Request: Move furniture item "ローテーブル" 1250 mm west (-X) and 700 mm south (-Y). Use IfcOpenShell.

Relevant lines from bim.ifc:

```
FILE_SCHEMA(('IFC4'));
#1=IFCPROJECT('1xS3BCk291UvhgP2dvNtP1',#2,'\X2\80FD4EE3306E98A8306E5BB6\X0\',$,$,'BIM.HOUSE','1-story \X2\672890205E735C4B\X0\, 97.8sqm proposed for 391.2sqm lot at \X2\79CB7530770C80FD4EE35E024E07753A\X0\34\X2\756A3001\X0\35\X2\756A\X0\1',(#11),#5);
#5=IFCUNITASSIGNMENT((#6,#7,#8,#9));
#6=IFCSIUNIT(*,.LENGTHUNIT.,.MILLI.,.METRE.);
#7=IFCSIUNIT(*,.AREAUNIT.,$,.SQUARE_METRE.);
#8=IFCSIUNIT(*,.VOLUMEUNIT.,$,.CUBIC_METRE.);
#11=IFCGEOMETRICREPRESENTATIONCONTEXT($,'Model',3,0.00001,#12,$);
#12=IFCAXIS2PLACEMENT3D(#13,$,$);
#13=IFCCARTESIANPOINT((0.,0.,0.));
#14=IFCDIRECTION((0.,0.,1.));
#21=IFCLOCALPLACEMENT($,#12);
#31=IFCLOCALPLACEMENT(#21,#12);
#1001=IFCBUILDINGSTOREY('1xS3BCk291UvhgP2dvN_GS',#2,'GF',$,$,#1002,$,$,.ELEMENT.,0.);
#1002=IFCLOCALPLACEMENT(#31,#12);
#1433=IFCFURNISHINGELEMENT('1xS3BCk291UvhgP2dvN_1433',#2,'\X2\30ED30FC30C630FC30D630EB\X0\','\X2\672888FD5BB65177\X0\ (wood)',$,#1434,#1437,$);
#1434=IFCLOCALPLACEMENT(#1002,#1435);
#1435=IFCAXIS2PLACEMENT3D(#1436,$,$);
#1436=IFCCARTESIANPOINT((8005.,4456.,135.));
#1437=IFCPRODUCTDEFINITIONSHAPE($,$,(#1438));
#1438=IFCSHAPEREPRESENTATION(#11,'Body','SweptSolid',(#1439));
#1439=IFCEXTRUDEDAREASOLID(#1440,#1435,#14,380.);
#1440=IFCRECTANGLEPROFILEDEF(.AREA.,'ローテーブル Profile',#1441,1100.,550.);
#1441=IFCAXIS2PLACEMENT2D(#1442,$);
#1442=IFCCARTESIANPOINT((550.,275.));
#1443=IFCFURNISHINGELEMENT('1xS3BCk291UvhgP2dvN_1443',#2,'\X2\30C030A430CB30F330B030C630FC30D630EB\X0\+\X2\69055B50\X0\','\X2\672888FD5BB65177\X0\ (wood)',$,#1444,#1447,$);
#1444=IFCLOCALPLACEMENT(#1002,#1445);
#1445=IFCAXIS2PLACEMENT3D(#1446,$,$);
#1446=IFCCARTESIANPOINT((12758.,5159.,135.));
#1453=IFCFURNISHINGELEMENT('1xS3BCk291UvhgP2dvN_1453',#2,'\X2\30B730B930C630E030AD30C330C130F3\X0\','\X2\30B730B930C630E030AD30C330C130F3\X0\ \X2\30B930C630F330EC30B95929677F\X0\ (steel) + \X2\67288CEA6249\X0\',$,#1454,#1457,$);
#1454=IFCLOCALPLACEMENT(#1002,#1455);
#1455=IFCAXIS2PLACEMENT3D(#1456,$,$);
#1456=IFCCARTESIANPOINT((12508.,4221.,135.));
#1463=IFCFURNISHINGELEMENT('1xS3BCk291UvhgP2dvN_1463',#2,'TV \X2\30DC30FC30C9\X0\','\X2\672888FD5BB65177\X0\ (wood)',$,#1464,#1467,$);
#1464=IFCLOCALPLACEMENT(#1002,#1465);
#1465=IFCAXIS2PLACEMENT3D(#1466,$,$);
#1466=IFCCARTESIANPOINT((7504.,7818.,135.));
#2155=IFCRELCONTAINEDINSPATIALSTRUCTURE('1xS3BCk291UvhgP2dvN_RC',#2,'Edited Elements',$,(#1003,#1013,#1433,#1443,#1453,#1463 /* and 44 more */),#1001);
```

```python
import ifcopenshell
import ifcopenshell.api.geometry
import ifcopenshell.util.placement

model = ifcopenshell.open("bim.ifc")

item = model.by_guid("1xS3BCk291UvhgP2dvN_1433")
matrix = ifcopenshell.util.placement.get_local_placement(item.ObjectPlacement)
matrix[0, 3] -= 1250.0
matrix[1, 3] -= 700.0
ifcopenshell.api.geometry.edit_object_placement(model, product=item, matrix=matrix, is_si=False)

print(ifcopenshell.util.placement.get_local_placement(item.ObjectPlacement).round(3) + 0.0)

model.write("bim_rev.ifc")
```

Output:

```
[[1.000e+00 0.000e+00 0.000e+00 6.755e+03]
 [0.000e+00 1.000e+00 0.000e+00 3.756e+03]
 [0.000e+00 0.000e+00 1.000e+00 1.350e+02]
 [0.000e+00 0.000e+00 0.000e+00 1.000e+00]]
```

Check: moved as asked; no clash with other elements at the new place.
